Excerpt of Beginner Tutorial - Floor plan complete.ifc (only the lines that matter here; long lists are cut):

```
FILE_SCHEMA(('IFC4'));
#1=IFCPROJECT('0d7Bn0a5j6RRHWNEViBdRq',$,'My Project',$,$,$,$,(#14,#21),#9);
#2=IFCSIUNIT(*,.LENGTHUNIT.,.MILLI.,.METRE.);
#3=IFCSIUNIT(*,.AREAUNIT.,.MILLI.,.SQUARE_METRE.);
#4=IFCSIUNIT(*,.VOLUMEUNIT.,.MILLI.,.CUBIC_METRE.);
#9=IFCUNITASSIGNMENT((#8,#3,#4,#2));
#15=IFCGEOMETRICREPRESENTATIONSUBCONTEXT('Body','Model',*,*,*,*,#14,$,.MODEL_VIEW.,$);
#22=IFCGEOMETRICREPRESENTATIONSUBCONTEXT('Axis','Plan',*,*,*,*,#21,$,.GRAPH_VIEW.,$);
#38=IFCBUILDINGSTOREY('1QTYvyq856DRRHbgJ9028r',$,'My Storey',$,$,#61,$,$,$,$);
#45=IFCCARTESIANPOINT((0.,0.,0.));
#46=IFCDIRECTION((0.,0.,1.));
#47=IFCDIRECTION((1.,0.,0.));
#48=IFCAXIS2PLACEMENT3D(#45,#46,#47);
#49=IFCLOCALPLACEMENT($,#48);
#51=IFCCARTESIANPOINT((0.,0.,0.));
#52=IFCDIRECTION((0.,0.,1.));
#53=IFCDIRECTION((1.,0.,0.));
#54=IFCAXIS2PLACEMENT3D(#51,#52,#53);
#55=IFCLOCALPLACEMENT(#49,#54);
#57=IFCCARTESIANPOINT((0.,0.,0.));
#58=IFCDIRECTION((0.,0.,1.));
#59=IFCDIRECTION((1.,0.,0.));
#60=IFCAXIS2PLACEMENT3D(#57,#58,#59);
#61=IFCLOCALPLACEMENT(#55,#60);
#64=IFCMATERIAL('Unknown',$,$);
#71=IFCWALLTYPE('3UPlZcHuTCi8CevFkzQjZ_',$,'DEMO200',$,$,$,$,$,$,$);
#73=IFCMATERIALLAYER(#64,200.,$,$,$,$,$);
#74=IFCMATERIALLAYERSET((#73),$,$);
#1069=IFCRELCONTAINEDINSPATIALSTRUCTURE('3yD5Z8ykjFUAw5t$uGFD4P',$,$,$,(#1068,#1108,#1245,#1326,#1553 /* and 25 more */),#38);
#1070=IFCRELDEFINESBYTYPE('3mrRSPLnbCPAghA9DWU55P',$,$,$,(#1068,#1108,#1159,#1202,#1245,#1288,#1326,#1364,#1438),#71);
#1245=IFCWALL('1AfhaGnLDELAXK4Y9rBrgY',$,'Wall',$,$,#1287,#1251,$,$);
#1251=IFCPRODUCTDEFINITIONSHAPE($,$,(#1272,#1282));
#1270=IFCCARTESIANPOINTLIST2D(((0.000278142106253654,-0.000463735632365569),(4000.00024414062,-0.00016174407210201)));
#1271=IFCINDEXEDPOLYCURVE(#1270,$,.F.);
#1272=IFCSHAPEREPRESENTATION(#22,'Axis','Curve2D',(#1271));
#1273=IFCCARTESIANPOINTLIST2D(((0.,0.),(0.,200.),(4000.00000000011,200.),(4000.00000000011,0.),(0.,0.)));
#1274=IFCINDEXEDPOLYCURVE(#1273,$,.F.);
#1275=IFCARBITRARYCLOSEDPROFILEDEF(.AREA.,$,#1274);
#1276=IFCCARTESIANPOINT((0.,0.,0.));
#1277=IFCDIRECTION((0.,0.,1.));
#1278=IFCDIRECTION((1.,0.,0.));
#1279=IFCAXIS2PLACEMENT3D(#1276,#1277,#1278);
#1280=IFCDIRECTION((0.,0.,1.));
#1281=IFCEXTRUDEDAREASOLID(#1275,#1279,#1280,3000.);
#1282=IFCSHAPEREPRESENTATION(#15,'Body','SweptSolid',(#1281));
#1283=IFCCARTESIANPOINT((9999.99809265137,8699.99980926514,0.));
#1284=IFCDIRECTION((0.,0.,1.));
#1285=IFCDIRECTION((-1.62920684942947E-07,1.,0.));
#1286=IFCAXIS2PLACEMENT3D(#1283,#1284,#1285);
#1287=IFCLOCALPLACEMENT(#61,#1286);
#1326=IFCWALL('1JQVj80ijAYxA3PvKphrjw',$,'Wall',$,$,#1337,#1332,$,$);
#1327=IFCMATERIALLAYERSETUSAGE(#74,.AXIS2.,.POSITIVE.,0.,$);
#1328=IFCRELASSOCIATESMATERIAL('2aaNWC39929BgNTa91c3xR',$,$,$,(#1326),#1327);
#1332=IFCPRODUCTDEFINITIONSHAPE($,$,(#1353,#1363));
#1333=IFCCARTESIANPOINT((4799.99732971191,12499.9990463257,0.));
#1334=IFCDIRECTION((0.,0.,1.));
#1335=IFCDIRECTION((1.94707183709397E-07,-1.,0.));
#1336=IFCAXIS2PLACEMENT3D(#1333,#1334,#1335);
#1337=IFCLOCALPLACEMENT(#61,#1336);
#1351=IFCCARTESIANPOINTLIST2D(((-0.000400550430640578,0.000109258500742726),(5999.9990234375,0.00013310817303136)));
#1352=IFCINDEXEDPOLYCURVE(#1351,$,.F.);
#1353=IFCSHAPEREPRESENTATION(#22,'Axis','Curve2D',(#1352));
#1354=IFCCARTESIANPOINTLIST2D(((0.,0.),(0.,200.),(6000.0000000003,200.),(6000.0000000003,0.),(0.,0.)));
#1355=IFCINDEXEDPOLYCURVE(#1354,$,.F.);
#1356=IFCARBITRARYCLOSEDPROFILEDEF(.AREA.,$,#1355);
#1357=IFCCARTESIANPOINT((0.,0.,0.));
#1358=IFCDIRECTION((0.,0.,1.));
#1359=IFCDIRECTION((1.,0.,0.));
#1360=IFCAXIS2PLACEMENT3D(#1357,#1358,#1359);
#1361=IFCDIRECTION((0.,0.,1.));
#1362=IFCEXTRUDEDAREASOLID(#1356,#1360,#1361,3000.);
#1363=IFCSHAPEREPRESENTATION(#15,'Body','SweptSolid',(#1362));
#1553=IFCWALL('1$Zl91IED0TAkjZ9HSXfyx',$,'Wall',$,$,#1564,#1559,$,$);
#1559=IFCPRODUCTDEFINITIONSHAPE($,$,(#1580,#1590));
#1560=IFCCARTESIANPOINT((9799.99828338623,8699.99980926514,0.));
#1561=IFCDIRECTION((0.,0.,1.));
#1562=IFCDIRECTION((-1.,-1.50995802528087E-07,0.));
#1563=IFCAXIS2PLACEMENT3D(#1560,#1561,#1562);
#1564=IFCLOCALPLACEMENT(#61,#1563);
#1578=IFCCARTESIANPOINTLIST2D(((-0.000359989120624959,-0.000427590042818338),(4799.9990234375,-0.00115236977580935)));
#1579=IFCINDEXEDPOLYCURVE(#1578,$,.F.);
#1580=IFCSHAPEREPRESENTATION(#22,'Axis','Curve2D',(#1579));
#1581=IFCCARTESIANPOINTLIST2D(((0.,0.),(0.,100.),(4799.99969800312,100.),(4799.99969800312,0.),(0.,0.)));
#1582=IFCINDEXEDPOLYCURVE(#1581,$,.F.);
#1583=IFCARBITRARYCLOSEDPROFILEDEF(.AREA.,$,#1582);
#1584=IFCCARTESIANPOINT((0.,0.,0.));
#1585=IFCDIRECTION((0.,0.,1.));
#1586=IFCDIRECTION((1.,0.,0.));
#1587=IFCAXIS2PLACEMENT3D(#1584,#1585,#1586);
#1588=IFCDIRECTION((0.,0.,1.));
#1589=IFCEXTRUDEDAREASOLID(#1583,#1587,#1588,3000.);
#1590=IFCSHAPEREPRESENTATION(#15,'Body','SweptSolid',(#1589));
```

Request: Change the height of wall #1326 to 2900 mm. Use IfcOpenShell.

```python
import ifcopenshell
import ifcopenshell.geom
import ifcopenshell.util.representation
import ifcopenshell.util.shape
import ifcopenshell.util.unit

model = ifcopenshell.open("Beginner Tutorial - Floor plan complete.ifc")
unit_scale = ifcopenshell.util.unit.calculate_unit_scale(model)
settings = ifcopenshell.geom.settings()


def volume(element):
    """Net volume in cubic metres, openings subtracted."""
    shape = ifcopenshell.geom.create_shape(settings, element)
    return ifcopenshell.util.shape.get_volume(shape.geometry)


wall = model.by_guid("1JQVj80ijAYxA3PvKphrjw")
before = volume(wall)

body = ifcopenshell.util.representation.get_representation(wall, "Model", "Body")
solid = body.Items[0]
old_height = solid.Depth
solid.Depth = 2.9 / unit_scale
after = volume(wall)

print(f"height {old_height:g} -> {solid.Depth:g}, volume {before:.3f} -> {after:.3f} m3")

model.write("Beginner Tutorial - Floor plan complete_updated.ifc")
```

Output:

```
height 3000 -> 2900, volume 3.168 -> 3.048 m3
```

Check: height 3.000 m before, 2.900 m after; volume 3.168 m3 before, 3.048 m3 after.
